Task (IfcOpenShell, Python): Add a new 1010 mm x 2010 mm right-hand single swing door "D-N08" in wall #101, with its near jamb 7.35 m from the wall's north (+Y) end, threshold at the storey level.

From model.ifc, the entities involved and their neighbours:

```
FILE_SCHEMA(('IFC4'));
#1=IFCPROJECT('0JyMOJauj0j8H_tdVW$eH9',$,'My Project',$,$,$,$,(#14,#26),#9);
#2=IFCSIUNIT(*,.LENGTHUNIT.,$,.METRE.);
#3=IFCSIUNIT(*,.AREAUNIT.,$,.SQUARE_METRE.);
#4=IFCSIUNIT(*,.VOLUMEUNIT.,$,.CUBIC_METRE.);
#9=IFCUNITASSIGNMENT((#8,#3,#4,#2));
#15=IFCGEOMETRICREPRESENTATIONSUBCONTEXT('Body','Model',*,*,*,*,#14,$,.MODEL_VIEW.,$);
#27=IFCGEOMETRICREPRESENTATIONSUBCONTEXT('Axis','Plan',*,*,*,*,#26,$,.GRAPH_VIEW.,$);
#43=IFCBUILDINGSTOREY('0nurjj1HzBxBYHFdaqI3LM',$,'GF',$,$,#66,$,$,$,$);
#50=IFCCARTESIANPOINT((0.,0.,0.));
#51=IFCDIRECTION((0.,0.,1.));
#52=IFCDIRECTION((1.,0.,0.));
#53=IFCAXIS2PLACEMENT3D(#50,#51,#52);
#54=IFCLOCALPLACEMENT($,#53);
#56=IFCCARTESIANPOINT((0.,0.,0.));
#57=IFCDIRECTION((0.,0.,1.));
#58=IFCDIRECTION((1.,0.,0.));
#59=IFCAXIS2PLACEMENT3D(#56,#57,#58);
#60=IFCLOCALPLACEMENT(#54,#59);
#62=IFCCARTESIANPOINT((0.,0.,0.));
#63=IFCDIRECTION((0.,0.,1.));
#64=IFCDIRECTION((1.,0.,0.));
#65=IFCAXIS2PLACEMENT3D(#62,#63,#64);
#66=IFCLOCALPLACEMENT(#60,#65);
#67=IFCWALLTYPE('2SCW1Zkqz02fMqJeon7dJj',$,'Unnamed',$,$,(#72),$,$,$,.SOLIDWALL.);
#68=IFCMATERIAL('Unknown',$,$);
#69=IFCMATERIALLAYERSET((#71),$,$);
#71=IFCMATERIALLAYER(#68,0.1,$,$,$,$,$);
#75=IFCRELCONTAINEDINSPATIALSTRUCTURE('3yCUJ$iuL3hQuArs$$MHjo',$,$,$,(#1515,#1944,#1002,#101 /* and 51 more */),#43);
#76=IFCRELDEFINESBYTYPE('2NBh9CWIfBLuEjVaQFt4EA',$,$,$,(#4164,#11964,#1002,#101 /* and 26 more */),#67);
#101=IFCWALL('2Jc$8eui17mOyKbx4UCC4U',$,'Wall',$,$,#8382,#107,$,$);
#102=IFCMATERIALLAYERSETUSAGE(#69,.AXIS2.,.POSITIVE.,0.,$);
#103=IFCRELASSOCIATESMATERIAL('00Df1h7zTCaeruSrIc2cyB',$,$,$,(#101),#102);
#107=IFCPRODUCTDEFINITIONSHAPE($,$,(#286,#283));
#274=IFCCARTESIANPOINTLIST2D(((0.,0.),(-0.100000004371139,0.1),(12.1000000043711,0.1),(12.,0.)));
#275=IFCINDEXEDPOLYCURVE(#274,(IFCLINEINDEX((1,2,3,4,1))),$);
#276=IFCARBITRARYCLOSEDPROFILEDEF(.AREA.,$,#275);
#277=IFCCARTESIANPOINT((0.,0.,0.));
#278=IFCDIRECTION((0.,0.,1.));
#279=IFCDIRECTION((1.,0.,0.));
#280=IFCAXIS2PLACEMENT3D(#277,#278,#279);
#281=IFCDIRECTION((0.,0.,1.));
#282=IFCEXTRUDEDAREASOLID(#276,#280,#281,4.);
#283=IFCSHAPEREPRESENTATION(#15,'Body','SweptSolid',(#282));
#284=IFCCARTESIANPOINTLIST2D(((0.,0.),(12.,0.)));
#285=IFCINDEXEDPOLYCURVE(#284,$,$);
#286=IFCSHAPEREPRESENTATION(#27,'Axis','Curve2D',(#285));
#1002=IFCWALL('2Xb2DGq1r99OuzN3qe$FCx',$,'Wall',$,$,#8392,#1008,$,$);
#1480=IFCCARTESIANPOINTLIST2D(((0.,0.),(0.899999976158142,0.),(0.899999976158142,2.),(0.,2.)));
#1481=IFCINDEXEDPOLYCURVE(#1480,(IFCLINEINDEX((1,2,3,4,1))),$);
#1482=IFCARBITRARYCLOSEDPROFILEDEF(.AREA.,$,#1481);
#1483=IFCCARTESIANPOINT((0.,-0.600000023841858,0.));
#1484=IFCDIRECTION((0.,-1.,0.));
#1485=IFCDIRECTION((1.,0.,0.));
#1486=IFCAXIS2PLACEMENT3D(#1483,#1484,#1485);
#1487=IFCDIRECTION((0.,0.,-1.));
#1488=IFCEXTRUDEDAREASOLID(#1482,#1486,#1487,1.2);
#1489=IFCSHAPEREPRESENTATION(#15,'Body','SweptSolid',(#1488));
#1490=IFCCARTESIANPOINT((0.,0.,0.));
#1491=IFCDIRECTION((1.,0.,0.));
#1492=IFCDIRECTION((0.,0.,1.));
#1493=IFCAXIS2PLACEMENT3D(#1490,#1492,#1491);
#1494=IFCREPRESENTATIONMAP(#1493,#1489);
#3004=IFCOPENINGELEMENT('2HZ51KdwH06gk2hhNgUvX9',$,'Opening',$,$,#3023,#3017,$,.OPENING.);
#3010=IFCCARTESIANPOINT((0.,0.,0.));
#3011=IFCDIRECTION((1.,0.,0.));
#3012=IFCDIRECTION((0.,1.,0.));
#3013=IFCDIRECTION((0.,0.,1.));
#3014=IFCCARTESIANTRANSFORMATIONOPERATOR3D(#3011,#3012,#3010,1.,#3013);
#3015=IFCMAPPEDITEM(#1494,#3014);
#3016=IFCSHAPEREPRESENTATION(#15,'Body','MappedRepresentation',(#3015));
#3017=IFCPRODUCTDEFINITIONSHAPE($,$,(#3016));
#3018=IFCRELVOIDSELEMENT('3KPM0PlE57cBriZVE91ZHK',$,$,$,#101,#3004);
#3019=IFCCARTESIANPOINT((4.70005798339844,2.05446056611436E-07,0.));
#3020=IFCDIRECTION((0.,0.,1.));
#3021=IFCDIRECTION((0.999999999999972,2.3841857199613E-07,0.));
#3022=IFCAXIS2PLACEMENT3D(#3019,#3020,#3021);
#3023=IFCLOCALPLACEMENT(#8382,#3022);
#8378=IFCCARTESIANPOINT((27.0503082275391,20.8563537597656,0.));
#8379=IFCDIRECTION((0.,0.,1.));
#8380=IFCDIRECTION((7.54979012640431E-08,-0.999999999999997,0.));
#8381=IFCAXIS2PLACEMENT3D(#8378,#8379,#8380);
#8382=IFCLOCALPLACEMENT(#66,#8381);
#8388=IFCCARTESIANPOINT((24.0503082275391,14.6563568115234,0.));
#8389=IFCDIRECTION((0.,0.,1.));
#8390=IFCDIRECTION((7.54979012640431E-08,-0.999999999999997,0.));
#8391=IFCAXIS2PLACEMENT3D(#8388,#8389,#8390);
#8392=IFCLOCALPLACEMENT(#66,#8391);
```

```python
import numpy as np
import ifcopenshell
import ifcopenshell.api.feature
import ifcopenshell.api.geometry
import ifcopenshell.api.root
import ifcopenshell.api.spatial
import ifcopenshell.geom
import ifcopenshell.util.element
import ifcopenshell.util.placement
import ifcopenshell.util.representation
import ifcopenshell.util.shape
import ifcopenshell.util.unit

model = ifcopenshell.open("model.ifc")
unit_scale = ifcopenshell.util.unit.calculate_unit_scale(model)
settings = ifcopenshell.geom.settings()


def volume(element):
    """Net volume in cubic metres, openings subtracted."""
    shape = ifcopenshell.geom.create_shape(settings, element)
    return ifcopenshell.util.shape.get_volume(shape.geometry)


wall = model.by_guid("2Jc$8eui17mOyKbx4UCC4U")
storey = ifcopenshell.util.element.get_container(wall, ifc_class="IfcBuildingStorey")
context = ifcopenshell.util.representation.get_context(model, "Model", "Body", "MODEL_VIEW")
before = volume(wall)

width, height, from_end, sill = 1.01, 2.01, 7.35, 0.0  # metres

# The wall runs along its own X axis, and the end named is its -X end.
wall_shape = ifcopenshell.geom.create_shape(settings, wall)
x, y, z = ifcopenshell.util.shape.get_vertices(wall_shape.geometry).T
start = x.min() + from_end
face, thickness = float(y.min()), float(y.max() - y.min())
wall_matrix = ifcopenshell.util.placement.get_local_placement(wall.ObjectPlacement)
level = ifcopenshell.util.placement.get_local_placement(storey.ObjectPlacement)[2, 3]


def in_wall(x, y):
    """Placement at x, y metres in the wall's axes, at sill height."""
    matrix = wall_matrix.copy()
    matrix[:, 3] = wall_matrix @ np.array([x / unit_scale, y / unit_scale, 0.0, 1.0])
    matrix[2, 3] = level + sill / unit_scale
    return matrix


# Opening: a box that overshoots both wall faces by 50 mm.
opening = ifcopenshell.api.root.create_entity(model, ifc_class="IfcOpeningElement", predefined_type="OPENING")
box = ifcopenshell.api.geometry.add_wall_representation(
    model, context=context, length=width, height=height, thickness=thickness + 0.1
)
ifcopenshell.api.geometry.assign_representation(model, product=opening, representation=box)
ifcopenshell.api.geometry.edit_object_placement(model, product=opening, matrix=in_wall(start, face - 0.05), is_si=False)
ifcopenshell.api.feature.add_feature(model, feature=opening, element=wall)

door = ifcopenshell.api.root.create_entity(model, ifc_class="IfcDoor", name="D-N08", predefined_type="DOOR")
door.OverallWidth, door.OverallHeight = width / unit_scale, height / unit_scale
door.OperationType = "SINGLE_SWING_RIGHT"
body = ifcopenshell.api.geometry.add_door_representation(
    model,
    context=context,
    overall_width=door.OverallWidth,
    overall_height=door.OverallHeight,
    operation_type="SINGLE_SWING_RIGHT",
    lining_properties={"LiningDepth": thickness / unit_scale, "ThresholdDepth": thickness / unit_scale},
)
ifcopenshell.api.geometry.assign_representation(model, product=door, representation=body)
ifcopenshell.api.spatial.assign_container(model, products=[door], relating_structure=storey)
ifcopenshell.api.feature.add_filling(model, opening=opening, element=door)

# The lining spans the wall, so the door starts at the wall face.
ifcopenshell.api.geometry.edit_object_placement(model, product=door, matrix=in_wall(start, face), is_si=False)

after = volume(wall)

print(f"wall volume {before:.3f} -> {after:.3f} m3")

model.write("model_updated.ifc")
```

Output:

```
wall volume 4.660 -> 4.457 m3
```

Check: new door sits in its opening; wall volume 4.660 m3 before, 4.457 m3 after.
